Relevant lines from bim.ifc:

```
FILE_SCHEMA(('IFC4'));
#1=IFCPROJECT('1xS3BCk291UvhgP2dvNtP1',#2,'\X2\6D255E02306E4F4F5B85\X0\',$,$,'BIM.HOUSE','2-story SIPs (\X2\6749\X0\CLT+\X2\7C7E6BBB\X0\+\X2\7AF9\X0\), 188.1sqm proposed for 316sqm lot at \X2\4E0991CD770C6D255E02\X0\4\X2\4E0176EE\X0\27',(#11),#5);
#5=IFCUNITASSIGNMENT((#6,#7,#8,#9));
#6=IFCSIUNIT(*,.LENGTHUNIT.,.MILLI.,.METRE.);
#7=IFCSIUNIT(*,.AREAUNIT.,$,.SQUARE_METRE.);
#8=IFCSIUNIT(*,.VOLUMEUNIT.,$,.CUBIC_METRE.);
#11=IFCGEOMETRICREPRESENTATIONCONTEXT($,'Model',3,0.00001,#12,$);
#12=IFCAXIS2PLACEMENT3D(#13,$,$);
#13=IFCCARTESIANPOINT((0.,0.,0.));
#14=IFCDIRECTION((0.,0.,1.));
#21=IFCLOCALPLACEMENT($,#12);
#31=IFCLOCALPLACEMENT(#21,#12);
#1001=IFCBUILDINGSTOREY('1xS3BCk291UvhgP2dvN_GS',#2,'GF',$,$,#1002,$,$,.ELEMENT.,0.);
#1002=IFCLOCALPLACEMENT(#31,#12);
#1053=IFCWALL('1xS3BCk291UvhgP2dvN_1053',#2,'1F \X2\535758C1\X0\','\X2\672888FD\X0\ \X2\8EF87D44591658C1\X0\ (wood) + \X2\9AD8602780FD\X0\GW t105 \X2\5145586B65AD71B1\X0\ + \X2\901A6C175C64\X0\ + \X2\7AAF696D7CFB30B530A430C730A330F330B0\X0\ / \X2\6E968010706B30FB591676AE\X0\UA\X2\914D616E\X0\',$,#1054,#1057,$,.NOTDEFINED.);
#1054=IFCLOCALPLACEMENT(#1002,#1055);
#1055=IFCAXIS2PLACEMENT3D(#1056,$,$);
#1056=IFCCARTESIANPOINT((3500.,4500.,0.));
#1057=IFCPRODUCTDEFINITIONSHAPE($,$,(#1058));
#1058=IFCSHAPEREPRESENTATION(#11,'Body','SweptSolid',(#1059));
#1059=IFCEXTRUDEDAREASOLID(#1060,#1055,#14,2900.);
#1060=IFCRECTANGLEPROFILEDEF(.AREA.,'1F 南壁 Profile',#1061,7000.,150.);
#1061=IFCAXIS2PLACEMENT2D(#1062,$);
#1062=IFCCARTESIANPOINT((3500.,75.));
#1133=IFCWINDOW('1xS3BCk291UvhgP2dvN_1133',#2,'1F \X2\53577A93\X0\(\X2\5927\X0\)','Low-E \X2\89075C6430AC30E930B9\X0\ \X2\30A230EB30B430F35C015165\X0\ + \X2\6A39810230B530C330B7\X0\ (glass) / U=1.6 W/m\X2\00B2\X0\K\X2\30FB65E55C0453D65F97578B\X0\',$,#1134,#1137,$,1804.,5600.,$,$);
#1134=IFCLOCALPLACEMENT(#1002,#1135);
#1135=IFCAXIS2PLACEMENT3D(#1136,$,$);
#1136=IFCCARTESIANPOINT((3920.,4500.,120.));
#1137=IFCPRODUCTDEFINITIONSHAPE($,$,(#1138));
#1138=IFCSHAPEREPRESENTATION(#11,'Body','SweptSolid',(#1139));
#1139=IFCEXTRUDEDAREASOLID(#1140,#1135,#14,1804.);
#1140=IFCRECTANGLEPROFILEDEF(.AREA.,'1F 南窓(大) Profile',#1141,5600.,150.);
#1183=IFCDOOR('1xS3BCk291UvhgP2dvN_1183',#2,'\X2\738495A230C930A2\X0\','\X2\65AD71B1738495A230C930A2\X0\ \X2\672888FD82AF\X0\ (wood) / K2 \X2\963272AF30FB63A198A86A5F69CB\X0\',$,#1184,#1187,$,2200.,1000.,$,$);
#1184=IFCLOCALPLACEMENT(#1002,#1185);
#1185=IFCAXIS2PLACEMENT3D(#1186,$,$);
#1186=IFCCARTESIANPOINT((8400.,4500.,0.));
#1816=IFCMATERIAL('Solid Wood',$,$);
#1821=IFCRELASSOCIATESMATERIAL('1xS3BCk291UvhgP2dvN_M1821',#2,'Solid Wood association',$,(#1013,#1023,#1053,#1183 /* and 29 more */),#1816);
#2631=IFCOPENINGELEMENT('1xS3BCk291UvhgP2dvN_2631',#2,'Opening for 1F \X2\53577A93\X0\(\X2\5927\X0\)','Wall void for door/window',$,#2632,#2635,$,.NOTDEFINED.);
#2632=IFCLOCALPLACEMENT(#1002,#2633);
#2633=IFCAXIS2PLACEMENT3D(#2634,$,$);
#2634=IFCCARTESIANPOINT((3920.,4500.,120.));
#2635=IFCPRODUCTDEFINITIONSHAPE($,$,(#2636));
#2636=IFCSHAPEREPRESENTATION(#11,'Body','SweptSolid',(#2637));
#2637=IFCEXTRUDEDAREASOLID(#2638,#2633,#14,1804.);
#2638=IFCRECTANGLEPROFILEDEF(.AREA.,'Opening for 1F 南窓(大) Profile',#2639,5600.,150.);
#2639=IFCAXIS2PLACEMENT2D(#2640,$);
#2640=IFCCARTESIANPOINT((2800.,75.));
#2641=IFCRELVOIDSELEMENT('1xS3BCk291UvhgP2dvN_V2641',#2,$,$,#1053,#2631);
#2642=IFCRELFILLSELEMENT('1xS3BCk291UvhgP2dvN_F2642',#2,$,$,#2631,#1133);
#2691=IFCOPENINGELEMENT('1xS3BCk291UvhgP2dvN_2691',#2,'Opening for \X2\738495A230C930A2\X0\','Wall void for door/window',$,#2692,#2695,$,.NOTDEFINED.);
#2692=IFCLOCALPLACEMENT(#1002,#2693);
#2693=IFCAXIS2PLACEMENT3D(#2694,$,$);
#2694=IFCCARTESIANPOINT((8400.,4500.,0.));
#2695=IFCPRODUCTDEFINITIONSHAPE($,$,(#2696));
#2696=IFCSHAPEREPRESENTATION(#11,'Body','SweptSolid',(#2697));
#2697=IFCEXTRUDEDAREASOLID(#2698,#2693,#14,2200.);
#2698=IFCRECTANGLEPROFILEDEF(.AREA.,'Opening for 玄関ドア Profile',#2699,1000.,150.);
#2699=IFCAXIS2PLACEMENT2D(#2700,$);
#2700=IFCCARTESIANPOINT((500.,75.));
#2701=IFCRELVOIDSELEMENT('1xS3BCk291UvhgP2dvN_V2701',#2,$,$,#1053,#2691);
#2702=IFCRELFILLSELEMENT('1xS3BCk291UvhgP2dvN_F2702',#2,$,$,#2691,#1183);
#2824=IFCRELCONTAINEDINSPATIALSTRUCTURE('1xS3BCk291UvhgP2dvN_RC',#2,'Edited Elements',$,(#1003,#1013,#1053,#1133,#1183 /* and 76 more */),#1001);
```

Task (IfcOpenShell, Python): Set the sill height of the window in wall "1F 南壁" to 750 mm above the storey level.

```python
import numpy as np
import ifcopenshell
import ifcopenshell.api.geometry
import ifcopenshell.geom
import ifcopenshell.util.element
import ifcopenshell.util.placement
import ifcopenshell.util.shape
import ifcopenshell.util.unit

model = ifcopenshell.open("bim.ifc")
unit_scale = ifcopenshell.util.unit.calculate_unit_scale(model)

window = model.by_id(1133)
opening = window.FillsVoids[0].RelatingOpeningElement
storey = ifcopenshell.util.element.get_container(window, ifc_class="IfcBuildingStorey")
level = ifcopenshell.util.placement.get_local_placement(storey.ObjectPlacement)[2, 3]

# The opening's origin need not be at the sill, so measure its lowest point.
shape = ifcopenshell.geom.create_shape(ifcopenshell.geom.settings(), opening)
bottom = ifcopenshell.util.shape.get_shape_bottom_elevation(shape, shape.geometry) / unit_scale
dz = level + 750.0 - bottom

shift = np.array([0.0, 0.0, dz])
# The window is not placed relative to its opening, so move both.
for product in (opening, window):
    matrix = ifcopenshell.util.placement.get_local_placement(product.ObjectPlacement)
    matrix[:3, 3] += shift
    ifcopenshell.api.geometry.edit_object_placement(model, product=product, matrix=matrix, is_si=False)

print(f"moved by {dz * unit_scale:+.3f} m")

model.write("bim_v2.ifc")
```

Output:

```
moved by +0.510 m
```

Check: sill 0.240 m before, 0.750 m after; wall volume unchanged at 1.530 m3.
